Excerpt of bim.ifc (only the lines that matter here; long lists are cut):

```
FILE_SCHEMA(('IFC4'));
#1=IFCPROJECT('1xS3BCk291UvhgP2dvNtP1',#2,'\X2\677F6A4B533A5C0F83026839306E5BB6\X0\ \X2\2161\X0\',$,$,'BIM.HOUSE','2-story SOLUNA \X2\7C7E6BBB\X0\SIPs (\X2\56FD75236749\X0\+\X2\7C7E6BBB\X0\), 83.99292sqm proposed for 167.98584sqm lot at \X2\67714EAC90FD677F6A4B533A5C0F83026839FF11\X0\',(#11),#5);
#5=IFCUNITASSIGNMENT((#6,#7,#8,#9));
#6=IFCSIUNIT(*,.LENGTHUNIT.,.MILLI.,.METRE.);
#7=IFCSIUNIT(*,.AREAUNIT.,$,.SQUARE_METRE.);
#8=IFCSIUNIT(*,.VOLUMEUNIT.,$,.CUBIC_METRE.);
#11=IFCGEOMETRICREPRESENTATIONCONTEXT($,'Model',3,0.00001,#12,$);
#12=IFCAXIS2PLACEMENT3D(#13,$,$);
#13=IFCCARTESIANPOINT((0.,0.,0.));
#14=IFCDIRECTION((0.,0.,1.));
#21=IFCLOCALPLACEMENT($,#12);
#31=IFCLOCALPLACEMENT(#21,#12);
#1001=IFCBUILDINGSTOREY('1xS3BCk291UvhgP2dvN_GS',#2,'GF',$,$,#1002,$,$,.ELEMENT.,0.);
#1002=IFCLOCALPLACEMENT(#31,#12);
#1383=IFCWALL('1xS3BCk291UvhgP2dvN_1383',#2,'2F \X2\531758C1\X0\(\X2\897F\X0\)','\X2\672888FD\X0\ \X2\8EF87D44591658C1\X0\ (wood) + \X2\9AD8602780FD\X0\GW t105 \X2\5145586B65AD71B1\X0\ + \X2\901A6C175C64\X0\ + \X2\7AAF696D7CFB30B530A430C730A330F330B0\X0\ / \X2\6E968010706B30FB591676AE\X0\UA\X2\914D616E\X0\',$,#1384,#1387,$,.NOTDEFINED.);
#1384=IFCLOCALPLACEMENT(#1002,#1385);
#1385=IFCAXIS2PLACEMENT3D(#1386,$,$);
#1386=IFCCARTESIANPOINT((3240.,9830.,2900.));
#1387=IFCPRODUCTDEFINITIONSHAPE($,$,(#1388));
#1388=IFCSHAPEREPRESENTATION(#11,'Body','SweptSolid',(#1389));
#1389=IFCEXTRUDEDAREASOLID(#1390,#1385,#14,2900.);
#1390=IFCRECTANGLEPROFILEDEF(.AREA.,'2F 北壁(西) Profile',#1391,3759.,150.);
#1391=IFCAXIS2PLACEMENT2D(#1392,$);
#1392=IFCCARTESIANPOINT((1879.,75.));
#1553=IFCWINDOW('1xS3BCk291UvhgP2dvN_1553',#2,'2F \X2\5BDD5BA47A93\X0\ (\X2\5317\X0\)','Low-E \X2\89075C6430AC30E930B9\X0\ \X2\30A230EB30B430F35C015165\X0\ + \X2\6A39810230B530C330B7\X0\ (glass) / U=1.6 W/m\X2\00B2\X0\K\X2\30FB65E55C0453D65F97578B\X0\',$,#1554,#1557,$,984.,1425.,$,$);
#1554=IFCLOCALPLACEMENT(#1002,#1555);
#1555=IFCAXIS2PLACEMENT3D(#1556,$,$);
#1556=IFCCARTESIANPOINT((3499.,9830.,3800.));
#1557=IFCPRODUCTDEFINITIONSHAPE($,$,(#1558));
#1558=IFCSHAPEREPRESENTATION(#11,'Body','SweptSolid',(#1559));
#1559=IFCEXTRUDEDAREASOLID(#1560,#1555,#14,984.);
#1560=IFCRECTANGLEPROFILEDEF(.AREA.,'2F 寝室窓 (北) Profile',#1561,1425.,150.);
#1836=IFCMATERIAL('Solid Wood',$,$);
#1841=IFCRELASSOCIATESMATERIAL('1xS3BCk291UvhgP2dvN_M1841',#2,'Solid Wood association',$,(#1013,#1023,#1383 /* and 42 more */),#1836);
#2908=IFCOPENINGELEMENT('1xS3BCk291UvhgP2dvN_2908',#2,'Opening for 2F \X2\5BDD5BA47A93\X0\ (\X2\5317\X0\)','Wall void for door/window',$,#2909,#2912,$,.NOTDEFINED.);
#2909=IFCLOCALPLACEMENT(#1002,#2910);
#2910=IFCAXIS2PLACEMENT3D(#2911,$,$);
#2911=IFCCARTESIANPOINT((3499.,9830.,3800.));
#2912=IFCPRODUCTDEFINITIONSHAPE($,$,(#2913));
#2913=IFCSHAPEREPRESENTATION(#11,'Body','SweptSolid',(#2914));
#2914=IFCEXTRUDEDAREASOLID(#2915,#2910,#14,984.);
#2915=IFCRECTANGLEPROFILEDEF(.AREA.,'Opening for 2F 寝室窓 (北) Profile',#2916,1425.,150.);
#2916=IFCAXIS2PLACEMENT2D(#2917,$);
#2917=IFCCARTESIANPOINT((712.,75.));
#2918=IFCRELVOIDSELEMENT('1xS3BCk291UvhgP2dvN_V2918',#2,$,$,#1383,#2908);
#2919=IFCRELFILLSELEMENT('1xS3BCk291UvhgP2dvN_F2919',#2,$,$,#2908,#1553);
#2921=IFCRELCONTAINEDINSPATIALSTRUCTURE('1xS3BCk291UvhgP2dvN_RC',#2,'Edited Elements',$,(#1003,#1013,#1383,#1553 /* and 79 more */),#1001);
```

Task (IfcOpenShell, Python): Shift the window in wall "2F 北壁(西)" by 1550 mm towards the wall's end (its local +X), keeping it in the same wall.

```python
import ifcopenshell
import ifcopenshell.api.geometry
import ifcopenshell.util.placement

model = ifcopenshell.open("bim.ifc")

window = model.by_guid("1xS3BCk291UvhgP2dvN_1553")
opening = window.FillsVoids[0].RelatingOpeningElement
wall = opening.VoidsElements[0].RelatingBuildingElement

wall_matrix = ifcopenshell.util.placement.get_local_placement(wall.ObjectPlacement)
shift = wall_matrix[:3, 0] * 1550.0
before = ifcopenshell.util.placement.get_local_placement(window.ObjectPlacement)[:3, 3].copy()

# The window is not placed relative to its opening, so move both.
for product in (opening, window):
    matrix = ifcopenshell.util.placement.get_local_placement(product.ObjectPlacement)
    matrix[:3, 3] += shift
    ifcopenshell.api.geometry.edit_object_placement(model, product=product, matrix=matrix, is_si=False)

after = ifcopenshell.util.placement.get_local_placement(window.ObjectPlacement)[:3, 3]
print("window moved by", (after - before).round(3) + 0.0)

model.write("bim_v2.ifc")
```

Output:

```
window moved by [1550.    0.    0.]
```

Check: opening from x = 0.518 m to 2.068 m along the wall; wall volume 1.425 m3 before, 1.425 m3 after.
